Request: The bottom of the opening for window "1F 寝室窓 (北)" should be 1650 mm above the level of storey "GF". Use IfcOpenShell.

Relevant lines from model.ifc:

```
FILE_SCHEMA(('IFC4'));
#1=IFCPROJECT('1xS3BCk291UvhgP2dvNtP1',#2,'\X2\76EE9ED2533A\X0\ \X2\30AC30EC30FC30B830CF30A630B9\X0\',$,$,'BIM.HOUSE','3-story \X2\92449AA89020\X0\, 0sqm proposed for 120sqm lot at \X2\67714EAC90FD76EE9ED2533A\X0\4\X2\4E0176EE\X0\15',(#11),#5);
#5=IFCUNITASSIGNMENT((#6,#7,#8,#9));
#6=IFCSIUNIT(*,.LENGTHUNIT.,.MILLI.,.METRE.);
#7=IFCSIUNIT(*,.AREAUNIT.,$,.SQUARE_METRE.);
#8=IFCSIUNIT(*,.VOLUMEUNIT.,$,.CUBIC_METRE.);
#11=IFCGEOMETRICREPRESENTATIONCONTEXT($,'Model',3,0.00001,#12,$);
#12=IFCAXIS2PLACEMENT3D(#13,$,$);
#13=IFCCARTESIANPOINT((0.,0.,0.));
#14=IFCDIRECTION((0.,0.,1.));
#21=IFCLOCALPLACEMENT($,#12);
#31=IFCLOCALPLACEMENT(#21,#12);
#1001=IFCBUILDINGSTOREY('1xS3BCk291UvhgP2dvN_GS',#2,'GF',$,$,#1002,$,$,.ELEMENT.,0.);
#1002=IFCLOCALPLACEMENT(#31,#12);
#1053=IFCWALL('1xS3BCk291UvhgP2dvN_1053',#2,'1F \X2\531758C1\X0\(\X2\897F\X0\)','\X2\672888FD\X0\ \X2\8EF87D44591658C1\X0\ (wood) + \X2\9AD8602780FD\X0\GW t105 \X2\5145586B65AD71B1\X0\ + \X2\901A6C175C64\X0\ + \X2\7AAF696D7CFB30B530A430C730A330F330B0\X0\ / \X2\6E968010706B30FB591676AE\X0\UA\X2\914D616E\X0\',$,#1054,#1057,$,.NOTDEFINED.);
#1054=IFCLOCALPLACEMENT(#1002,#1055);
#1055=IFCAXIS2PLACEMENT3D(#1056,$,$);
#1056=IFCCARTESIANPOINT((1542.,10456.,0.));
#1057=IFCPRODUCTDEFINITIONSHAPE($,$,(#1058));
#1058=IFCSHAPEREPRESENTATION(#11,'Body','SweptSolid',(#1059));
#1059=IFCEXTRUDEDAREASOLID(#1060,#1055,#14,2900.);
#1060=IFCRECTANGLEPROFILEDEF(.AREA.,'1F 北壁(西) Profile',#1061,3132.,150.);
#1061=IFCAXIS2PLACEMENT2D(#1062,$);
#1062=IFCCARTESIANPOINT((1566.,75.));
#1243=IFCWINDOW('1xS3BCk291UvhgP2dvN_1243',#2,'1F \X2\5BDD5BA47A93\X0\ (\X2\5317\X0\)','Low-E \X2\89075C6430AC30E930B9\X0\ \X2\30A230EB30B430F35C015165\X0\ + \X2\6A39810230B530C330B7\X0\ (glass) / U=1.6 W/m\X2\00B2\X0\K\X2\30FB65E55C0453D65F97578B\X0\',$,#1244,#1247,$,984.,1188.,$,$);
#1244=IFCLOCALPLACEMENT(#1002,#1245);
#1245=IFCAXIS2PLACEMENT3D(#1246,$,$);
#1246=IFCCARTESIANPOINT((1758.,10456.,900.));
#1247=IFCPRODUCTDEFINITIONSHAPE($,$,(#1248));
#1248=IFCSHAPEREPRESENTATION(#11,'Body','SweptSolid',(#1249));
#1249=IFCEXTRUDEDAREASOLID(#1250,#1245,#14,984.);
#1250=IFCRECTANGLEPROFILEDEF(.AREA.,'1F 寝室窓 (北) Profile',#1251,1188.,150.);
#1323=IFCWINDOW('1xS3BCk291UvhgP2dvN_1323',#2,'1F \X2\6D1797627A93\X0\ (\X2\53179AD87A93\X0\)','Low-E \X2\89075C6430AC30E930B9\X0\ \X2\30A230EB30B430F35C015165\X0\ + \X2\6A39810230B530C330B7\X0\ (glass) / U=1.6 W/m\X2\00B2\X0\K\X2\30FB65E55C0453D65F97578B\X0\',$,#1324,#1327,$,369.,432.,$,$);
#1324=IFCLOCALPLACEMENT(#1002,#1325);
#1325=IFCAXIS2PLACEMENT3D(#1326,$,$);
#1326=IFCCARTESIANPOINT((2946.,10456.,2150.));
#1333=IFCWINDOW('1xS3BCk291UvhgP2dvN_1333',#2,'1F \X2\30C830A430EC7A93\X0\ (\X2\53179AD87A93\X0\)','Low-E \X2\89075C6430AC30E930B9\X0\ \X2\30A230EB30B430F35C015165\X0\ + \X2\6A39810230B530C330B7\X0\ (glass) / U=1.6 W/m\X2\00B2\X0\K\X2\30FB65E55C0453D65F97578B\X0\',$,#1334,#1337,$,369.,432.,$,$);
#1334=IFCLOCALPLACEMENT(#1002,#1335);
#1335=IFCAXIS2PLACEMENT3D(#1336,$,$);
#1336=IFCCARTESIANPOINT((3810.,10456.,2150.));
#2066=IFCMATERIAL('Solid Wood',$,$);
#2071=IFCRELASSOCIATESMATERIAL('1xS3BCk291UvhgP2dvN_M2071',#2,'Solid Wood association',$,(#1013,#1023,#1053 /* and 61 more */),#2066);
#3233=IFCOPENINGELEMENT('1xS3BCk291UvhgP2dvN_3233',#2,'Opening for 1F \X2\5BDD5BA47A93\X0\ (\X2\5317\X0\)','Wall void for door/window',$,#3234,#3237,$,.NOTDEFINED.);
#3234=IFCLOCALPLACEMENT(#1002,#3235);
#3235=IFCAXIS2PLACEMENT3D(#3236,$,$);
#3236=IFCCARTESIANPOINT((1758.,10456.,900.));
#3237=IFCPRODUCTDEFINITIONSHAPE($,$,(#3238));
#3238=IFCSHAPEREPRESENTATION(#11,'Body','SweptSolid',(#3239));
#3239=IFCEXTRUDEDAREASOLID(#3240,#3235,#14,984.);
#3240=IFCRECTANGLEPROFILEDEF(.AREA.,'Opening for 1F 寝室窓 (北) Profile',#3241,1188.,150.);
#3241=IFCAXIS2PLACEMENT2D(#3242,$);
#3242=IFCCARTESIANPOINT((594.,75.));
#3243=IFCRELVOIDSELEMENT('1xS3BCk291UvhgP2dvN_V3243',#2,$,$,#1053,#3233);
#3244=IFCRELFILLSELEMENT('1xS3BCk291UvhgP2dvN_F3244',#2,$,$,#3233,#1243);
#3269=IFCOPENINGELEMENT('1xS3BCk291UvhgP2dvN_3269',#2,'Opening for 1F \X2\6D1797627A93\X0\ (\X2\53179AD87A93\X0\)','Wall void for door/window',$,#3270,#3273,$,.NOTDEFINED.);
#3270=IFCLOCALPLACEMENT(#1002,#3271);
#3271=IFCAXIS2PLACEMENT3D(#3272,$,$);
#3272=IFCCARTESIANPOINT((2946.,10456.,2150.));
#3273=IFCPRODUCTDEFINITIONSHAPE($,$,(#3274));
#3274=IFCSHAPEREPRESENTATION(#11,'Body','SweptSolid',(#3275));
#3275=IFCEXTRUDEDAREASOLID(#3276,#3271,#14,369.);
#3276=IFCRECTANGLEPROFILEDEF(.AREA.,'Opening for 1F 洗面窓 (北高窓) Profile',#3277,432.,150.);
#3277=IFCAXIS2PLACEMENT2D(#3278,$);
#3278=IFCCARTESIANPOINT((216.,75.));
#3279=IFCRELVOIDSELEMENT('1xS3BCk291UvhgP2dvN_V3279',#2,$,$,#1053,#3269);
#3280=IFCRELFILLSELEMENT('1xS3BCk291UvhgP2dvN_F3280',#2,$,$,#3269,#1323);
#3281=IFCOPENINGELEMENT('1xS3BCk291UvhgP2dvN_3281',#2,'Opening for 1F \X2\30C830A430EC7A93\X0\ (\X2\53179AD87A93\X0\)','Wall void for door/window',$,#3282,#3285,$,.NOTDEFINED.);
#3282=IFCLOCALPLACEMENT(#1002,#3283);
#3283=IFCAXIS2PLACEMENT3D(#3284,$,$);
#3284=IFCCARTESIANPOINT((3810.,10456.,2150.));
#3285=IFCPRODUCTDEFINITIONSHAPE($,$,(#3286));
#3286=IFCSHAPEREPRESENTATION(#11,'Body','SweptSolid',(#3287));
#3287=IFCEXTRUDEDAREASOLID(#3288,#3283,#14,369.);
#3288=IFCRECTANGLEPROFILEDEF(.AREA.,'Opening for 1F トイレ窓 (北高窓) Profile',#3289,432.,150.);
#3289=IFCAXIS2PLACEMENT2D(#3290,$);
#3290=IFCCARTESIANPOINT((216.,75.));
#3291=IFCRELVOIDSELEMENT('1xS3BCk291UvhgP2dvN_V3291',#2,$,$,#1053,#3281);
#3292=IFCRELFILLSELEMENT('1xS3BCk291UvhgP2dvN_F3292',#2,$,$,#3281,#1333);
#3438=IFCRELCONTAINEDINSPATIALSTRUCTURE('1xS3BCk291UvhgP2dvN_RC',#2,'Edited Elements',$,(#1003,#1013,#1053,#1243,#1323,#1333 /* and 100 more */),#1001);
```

```python
import numpy as np
import ifcopenshell
import ifcopenshell.api.geometry
import ifcopenshell.geom
import ifcopenshell.util.element
import ifcopenshell.util.placement
import ifcopenshell.util.shape
import ifcopenshell.util.unit

model = ifcopenshell.open("model.ifc")
unit_scale = ifcopenshell.util.unit.calculate_unit_scale(model)

window = model.by_guid("1xS3BCk291UvhgP2dvN_1243")
opening = window.FillsVoids[0].RelatingOpeningElement
storey = ifcopenshell.util.element.get_container(window, ifc_class="IfcBuildingStorey")
level = ifcopenshell.util.placement.get_local_placement(storey.ObjectPlacement)[2, 3]

# The opening's origin need not be at the sill, so measure its lowest point.
shape = ifcopenshell.geom.create_shape(ifcopenshell.geom.settings(), opening)
bottom = ifcopenshell.util.shape.get_shape_bottom_elevation(shape, shape.geometry) / unit_scale
dz = level + 1.65 / unit_scale - bottom

shift = np.array([0.0, 0.0, dz])
# The window is not placed relative to its opening, so move both.
for product in (opening, window):
    matrix = ifcopenshell.util.placement.get_local_placement(product.ObjectPlacement)
    matrix[:3, 3] += shift
    ifcopenshell.api.geometry.edit_object_placement(model, product=product, matrix=matrix, is_si=False)

print(f"moved by {dz * unit_scale:+.3f} m")

model.write("model_updated.ifc")
```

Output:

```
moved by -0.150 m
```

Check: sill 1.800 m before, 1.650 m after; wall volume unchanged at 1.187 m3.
